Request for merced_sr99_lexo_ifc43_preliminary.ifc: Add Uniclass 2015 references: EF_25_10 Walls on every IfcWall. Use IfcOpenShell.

First a look at what the model holds.

```python
import ifcopenshell

model = ifcopenshell.open("merced_sr99_lexo_ifc43_preliminary.ifc")
print(model.schema)
print("classifications:", [c.Name for c in model.by_type("IfcClassification")])
for ifc_class in ("IfcDoor", "IfcRoof", "IfcStair", "IfcWall", "IfcWindow"):
    print(ifc_class, len(model.by_type(ifc_class)))
```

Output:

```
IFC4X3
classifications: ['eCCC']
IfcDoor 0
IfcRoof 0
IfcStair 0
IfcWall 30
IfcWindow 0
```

```python
import ifcopenshell
import ifcopenshell.api.classification

model = ifcopenshell.open("merced_sr99_lexo_ifc43_preliminary.ifc")

system = ifcopenshell.api.classification.add_classification(model, classification="Uniclass 2015")

codes = {
    "IfcWall": ("EF_25_10", "Walls"),
}
for ifc_class, (code, name) in codes.items():
    products = model.by_type(ifc_class)
    ifcopenshell.api.classification.add_reference(
        model, products=products, classification=system, identification=code, name=name
    )
    print(code, len(products))

model.write("merced_sr99_lexo_ifc43_preliminary_v2.ifc")
```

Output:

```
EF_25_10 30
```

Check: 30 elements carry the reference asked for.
